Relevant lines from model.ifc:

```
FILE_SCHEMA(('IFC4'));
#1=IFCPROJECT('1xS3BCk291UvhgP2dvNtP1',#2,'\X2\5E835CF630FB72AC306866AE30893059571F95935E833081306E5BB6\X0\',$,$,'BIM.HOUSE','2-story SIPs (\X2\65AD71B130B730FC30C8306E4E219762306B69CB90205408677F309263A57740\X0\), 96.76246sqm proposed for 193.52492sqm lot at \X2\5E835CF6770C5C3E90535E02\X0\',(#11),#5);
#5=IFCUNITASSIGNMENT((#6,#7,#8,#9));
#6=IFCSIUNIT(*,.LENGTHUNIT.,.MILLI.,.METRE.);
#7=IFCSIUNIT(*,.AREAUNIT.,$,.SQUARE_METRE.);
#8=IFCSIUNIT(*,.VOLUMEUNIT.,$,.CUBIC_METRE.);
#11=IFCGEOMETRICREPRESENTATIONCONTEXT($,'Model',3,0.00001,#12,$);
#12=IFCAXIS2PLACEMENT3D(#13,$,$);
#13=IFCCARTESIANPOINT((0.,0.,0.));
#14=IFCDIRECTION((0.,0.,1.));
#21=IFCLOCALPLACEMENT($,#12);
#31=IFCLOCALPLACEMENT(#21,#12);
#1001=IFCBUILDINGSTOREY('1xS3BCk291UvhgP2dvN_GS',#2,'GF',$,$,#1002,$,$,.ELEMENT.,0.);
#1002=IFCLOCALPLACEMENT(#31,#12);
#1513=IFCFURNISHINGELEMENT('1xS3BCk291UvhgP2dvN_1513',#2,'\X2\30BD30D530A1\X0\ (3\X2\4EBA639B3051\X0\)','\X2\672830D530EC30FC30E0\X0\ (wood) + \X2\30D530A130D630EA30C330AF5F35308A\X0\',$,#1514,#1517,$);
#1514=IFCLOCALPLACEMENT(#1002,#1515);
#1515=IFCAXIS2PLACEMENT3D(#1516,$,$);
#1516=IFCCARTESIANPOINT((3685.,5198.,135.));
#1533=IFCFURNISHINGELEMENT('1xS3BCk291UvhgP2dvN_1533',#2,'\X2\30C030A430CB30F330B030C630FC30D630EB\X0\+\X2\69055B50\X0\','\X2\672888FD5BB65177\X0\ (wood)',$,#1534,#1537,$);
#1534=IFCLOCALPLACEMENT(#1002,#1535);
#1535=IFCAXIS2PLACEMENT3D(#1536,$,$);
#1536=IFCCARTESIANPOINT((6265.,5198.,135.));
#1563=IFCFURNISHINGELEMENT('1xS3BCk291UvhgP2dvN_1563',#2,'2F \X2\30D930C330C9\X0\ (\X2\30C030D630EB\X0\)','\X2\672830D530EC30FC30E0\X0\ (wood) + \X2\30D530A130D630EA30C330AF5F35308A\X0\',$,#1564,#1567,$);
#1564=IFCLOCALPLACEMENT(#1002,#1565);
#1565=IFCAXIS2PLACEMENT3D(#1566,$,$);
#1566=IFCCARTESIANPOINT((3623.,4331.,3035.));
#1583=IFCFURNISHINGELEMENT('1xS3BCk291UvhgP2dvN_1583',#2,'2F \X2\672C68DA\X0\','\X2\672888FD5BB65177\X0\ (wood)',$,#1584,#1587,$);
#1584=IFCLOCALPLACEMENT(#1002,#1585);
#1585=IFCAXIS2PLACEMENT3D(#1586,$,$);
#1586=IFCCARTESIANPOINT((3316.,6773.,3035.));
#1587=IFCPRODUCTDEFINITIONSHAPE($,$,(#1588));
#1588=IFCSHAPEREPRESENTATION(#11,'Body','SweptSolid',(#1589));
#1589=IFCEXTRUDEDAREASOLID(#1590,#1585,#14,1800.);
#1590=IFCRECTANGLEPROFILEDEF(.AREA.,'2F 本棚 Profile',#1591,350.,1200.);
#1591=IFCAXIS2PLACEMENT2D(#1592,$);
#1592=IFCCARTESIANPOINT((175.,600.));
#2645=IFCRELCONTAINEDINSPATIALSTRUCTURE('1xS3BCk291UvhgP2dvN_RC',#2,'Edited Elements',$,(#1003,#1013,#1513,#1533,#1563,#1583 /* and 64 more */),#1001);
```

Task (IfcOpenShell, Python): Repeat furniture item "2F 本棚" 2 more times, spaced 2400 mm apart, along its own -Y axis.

```python
import ifcopenshell
import ifcopenshell.api.geometry
import ifcopenshell.api.root
import ifcopenshell.util.element
import ifcopenshell.util.placement

model = ifcopenshell.open("model.ifc")


def reuse_history(source, copy):
    """copy_class also copies each property set's owner history, people and application; keep the originals."""
    for rel in copy.IsDefinedBy:
        if rel.is_a("IfcRelDefinesByProperties") and (history := rel.RelatingPropertyDefinition.OwnerHistory):
            rel.RelatingPropertyDefinition.OwnerHistory = source.OwnerHistory
            ifcopenshell.util.element.remove_deep2(model, history)


source = model.by_id(1583)
base = ifcopenshell.util.placement.get_local_placement(source.ObjectPlacement)
step = -base[:3, 1] * 2400.0

for i in range(1, 3):
    copy = ifcopenshell.api.root.copy_class(model, product=source)
    copy.Representation = ifcopenshell.util.element.copy_deep(
        model, source.Representation, exclude=["IfcGeometricRepresentationContext", "IfcRepresentationMap"]
    )
    reuse_history(source, copy)
    matrix = base.copy()
    matrix[:3, 3] += i * step
    print("added at", matrix[:3, 3].round(3) + 0.0)
    ifcopenshell.api.geometry.edit_object_placement(model, product=copy, matrix=matrix, is_si=False)

model.write("model-out.ifc")
```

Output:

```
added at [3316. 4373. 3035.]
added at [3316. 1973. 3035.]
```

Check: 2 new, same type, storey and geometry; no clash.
